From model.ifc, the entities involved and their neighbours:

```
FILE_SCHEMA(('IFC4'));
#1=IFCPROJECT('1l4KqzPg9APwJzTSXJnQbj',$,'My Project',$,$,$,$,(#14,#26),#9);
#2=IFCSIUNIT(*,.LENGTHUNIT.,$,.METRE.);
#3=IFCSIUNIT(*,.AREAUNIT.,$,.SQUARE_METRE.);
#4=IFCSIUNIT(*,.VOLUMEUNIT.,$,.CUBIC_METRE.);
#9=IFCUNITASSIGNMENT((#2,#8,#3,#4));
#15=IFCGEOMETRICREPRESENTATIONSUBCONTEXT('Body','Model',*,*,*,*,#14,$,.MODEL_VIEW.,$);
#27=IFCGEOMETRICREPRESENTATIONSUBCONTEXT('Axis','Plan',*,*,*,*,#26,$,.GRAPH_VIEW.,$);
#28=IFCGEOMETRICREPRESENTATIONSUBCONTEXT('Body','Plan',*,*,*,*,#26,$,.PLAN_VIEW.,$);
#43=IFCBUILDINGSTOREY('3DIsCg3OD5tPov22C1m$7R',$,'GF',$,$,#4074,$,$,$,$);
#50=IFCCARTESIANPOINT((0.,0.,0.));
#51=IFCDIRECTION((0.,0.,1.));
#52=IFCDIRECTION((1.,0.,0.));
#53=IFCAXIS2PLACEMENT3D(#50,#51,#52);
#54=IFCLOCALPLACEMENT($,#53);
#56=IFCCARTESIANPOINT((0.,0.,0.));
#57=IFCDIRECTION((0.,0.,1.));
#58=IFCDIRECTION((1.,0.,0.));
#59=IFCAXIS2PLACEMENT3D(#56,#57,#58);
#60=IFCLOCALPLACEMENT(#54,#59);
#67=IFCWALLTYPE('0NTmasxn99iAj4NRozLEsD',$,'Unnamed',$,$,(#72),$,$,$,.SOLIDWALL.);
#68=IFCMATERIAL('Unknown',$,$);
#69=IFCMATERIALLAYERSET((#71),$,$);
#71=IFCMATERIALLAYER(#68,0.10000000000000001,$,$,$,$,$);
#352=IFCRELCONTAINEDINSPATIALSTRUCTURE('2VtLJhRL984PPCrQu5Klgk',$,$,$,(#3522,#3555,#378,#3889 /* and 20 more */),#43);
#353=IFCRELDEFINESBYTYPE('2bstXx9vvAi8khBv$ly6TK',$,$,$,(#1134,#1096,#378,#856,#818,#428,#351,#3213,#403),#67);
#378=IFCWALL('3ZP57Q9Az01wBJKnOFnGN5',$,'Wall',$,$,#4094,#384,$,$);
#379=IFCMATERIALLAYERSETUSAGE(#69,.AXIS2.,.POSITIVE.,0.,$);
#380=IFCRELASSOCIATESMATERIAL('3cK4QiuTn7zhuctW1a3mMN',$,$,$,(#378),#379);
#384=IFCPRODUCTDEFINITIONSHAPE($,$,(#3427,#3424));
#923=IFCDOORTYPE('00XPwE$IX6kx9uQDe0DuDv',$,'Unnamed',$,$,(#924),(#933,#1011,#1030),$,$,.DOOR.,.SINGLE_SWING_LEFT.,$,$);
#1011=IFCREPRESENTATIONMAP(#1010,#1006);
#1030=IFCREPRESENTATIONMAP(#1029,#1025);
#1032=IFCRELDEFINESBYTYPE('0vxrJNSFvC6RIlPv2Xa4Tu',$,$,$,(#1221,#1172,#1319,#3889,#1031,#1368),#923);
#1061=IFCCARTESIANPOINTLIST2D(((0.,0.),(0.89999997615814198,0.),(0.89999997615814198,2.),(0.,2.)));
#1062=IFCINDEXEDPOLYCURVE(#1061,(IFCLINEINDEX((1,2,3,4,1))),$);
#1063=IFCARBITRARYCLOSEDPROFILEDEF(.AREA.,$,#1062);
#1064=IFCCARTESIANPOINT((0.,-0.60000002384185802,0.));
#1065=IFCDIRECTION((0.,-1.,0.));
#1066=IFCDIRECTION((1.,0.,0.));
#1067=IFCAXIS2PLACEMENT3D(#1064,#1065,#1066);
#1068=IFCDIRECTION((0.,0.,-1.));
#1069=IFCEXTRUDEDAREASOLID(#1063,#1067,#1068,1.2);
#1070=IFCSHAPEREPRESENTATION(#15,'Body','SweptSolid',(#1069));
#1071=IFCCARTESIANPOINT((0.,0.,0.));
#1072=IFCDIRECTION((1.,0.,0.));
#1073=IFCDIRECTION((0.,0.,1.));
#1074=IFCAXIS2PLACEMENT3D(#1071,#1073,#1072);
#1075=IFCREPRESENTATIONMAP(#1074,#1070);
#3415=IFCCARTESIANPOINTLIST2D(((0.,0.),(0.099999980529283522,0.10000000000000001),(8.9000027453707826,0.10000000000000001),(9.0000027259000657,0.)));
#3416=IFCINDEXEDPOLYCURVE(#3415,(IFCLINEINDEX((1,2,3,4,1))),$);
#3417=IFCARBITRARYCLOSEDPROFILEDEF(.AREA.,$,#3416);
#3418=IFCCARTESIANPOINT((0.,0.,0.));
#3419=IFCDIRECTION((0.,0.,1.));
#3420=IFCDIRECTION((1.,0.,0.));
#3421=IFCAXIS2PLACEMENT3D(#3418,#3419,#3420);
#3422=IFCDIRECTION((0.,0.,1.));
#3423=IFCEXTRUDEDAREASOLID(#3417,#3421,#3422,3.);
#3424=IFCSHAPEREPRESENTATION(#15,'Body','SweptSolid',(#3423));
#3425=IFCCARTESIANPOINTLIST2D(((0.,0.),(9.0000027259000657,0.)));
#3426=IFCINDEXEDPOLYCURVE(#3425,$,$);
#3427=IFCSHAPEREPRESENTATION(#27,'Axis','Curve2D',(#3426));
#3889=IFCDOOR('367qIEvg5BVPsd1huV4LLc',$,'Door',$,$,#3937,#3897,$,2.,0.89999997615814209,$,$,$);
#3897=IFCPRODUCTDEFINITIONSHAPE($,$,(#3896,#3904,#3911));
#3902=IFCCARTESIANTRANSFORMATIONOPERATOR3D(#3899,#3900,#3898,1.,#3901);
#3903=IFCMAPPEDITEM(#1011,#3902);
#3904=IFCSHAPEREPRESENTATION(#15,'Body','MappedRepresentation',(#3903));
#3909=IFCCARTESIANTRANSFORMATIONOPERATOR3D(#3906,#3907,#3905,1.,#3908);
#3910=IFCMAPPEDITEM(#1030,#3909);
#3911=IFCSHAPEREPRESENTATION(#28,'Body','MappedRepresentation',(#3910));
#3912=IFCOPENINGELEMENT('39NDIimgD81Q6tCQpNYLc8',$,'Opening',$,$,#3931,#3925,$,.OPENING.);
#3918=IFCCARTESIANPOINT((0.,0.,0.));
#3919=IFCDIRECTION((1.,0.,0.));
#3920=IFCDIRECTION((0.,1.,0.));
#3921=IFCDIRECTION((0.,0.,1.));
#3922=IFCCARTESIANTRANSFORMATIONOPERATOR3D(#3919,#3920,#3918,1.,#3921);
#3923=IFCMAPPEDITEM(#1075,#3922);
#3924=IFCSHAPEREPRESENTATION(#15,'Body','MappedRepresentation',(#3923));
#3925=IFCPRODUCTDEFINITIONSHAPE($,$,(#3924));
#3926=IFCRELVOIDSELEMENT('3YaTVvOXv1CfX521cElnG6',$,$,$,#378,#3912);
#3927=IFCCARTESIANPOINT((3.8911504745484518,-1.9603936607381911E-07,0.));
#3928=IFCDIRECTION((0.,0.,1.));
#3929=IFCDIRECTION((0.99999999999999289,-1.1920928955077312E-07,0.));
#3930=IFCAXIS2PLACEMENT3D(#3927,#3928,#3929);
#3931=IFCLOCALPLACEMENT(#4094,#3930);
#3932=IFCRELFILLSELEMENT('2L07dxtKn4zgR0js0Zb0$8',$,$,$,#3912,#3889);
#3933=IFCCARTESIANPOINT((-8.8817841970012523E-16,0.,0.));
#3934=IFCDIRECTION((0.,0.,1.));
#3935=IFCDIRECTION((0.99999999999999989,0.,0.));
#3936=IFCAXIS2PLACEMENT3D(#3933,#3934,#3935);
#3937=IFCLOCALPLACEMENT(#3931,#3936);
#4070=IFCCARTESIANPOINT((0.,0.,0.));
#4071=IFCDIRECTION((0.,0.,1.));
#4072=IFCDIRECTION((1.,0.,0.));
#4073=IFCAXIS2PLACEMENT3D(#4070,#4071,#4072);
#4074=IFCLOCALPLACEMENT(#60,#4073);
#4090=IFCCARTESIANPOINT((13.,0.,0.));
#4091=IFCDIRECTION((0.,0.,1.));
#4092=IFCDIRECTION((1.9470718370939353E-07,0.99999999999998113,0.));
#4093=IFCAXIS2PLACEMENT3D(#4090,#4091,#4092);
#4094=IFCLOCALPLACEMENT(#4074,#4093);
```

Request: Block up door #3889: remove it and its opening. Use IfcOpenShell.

```python
import ifcopenshell
import ifcopenshell.api.feature
import ifcopenshell.api.root
import ifcopenshell.geom
import ifcopenshell.util.shape

model = ifcopenshell.open("model.ifc")
settings = ifcopenshell.geom.settings()


def volume(element):
    """Net volume in cubic metres, openings subtracted."""
    shape = ifcopenshell.geom.create_shape(settings, element)
    return ifcopenshell.util.shape.get_volume(shape.geometry)


door = model.by_guid("367qIEvg5BVPsd1huV4LLc")
opening = door.FillsVoids[0].RelatingOpeningElement
wall = opening.VoidsElements[0].RelatingBuildingElement
before = volume(wall)

ifcopenshell.api.root.remove_product(model, product=door)
ifcopenshell.api.feature.remove_feature(model, feature=opening)

after = volume(wall)

print(f"wall volume {before:.3f} -> {after:.3f} m3")

model.write("model_rev.ifc")
```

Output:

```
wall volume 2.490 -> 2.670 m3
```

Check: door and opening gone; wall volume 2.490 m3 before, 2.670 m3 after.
